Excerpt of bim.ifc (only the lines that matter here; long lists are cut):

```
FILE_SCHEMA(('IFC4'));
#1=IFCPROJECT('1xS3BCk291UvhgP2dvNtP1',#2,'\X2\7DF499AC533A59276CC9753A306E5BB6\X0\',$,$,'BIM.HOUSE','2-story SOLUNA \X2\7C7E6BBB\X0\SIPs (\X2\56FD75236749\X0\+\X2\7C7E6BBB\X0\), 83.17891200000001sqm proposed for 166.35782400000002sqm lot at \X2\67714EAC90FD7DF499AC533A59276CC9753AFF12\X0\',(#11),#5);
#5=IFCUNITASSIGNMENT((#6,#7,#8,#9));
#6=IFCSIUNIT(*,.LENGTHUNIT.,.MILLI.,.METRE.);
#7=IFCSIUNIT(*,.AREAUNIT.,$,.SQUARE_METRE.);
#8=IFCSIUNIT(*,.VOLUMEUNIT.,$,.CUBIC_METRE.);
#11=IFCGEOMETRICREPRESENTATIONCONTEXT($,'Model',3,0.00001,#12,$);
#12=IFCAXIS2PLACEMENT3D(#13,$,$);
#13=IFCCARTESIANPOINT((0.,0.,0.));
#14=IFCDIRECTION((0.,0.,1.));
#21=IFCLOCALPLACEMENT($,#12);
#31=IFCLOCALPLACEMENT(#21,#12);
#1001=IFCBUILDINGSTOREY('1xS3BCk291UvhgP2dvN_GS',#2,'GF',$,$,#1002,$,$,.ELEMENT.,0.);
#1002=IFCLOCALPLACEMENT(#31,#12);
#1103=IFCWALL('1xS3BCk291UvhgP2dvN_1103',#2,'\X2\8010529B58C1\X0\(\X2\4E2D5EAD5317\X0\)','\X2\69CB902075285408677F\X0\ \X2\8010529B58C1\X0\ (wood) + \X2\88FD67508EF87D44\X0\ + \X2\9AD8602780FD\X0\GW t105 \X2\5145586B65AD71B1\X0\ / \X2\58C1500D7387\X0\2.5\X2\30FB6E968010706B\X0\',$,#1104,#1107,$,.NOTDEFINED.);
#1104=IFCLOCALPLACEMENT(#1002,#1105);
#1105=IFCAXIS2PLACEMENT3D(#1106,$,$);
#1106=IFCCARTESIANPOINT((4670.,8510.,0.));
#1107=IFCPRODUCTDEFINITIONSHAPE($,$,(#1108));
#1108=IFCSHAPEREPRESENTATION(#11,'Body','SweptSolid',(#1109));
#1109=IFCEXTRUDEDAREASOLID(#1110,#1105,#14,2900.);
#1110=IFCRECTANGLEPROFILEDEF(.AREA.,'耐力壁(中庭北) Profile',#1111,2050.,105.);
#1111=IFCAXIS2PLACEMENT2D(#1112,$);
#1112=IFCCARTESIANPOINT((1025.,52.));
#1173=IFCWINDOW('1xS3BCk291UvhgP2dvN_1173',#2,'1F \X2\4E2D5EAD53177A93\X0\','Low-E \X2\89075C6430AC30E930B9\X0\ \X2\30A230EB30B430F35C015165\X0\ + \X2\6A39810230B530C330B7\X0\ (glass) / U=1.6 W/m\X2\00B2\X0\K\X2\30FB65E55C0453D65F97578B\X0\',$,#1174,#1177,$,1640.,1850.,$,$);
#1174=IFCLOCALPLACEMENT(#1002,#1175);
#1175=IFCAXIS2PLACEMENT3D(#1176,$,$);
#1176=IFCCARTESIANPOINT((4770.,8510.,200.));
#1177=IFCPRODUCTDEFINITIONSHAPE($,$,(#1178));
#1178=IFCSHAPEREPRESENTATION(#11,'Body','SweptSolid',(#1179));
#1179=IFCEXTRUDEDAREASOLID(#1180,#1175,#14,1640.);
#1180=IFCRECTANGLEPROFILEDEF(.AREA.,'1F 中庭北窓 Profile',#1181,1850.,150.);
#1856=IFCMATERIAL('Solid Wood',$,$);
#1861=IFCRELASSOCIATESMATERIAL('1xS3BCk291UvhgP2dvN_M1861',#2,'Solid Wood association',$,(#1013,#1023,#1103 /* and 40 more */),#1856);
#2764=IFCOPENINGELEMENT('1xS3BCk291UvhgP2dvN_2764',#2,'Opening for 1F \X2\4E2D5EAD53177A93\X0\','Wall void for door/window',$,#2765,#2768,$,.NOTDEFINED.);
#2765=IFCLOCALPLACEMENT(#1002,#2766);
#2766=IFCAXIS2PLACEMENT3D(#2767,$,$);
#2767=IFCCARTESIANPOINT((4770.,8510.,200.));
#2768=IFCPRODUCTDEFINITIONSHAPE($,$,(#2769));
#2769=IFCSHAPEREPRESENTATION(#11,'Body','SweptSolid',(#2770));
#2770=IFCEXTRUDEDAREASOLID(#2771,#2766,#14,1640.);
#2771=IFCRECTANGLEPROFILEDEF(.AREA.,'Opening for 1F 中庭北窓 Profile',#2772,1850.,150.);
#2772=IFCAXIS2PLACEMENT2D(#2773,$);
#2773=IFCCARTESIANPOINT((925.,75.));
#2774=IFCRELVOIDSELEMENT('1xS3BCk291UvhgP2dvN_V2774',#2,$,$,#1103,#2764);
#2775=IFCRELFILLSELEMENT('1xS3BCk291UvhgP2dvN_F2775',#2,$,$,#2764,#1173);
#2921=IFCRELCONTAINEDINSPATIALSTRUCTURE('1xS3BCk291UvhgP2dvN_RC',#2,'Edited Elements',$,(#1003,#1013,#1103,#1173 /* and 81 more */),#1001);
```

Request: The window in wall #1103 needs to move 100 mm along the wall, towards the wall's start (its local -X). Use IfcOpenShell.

```python
import ifcopenshell
import ifcopenshell.api.geometry
import ifcopenshell.util.placement

model = ifcopenshell.open("bim.ifc")

window = model.by_guid("1xS3BCk291UvhgP2dvN_1173")
opening = window.FillsVoids[0].RelatingOpeningElement
wall = opening.VoidsElements[0].RelatingBuildingElement

wall_matrix = ifcopenshell.util.placement.get_local_placement(wall.ObjectPlacement)
shift = wall_matrix[:3, 0] * -100.0
before = ifcopenshell.util.placement.get_local_placement(window.ObjectPlacement)[:3, 3].copy()

# The window is not placed relative to its opening, so move both.
for product in (opening, window):
    matrix = ifcopenshell.util.placement.get_local_placement(product.ObjectPlacement)
    matrix[:3, 3] += shift
    ifcopenshell.api.geometry.edit_object_placement(model, product=product, matrix=matrix, is_si=False)

after = ifcopenshell.util.placement.get_local_placement(window.ObjectPlacement)[:3, 3]
print("window moved by", (after - before).round(3) + 0.0)

model.write("bim_rev.ifc")
```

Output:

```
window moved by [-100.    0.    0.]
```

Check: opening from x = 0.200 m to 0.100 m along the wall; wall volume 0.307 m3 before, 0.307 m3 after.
